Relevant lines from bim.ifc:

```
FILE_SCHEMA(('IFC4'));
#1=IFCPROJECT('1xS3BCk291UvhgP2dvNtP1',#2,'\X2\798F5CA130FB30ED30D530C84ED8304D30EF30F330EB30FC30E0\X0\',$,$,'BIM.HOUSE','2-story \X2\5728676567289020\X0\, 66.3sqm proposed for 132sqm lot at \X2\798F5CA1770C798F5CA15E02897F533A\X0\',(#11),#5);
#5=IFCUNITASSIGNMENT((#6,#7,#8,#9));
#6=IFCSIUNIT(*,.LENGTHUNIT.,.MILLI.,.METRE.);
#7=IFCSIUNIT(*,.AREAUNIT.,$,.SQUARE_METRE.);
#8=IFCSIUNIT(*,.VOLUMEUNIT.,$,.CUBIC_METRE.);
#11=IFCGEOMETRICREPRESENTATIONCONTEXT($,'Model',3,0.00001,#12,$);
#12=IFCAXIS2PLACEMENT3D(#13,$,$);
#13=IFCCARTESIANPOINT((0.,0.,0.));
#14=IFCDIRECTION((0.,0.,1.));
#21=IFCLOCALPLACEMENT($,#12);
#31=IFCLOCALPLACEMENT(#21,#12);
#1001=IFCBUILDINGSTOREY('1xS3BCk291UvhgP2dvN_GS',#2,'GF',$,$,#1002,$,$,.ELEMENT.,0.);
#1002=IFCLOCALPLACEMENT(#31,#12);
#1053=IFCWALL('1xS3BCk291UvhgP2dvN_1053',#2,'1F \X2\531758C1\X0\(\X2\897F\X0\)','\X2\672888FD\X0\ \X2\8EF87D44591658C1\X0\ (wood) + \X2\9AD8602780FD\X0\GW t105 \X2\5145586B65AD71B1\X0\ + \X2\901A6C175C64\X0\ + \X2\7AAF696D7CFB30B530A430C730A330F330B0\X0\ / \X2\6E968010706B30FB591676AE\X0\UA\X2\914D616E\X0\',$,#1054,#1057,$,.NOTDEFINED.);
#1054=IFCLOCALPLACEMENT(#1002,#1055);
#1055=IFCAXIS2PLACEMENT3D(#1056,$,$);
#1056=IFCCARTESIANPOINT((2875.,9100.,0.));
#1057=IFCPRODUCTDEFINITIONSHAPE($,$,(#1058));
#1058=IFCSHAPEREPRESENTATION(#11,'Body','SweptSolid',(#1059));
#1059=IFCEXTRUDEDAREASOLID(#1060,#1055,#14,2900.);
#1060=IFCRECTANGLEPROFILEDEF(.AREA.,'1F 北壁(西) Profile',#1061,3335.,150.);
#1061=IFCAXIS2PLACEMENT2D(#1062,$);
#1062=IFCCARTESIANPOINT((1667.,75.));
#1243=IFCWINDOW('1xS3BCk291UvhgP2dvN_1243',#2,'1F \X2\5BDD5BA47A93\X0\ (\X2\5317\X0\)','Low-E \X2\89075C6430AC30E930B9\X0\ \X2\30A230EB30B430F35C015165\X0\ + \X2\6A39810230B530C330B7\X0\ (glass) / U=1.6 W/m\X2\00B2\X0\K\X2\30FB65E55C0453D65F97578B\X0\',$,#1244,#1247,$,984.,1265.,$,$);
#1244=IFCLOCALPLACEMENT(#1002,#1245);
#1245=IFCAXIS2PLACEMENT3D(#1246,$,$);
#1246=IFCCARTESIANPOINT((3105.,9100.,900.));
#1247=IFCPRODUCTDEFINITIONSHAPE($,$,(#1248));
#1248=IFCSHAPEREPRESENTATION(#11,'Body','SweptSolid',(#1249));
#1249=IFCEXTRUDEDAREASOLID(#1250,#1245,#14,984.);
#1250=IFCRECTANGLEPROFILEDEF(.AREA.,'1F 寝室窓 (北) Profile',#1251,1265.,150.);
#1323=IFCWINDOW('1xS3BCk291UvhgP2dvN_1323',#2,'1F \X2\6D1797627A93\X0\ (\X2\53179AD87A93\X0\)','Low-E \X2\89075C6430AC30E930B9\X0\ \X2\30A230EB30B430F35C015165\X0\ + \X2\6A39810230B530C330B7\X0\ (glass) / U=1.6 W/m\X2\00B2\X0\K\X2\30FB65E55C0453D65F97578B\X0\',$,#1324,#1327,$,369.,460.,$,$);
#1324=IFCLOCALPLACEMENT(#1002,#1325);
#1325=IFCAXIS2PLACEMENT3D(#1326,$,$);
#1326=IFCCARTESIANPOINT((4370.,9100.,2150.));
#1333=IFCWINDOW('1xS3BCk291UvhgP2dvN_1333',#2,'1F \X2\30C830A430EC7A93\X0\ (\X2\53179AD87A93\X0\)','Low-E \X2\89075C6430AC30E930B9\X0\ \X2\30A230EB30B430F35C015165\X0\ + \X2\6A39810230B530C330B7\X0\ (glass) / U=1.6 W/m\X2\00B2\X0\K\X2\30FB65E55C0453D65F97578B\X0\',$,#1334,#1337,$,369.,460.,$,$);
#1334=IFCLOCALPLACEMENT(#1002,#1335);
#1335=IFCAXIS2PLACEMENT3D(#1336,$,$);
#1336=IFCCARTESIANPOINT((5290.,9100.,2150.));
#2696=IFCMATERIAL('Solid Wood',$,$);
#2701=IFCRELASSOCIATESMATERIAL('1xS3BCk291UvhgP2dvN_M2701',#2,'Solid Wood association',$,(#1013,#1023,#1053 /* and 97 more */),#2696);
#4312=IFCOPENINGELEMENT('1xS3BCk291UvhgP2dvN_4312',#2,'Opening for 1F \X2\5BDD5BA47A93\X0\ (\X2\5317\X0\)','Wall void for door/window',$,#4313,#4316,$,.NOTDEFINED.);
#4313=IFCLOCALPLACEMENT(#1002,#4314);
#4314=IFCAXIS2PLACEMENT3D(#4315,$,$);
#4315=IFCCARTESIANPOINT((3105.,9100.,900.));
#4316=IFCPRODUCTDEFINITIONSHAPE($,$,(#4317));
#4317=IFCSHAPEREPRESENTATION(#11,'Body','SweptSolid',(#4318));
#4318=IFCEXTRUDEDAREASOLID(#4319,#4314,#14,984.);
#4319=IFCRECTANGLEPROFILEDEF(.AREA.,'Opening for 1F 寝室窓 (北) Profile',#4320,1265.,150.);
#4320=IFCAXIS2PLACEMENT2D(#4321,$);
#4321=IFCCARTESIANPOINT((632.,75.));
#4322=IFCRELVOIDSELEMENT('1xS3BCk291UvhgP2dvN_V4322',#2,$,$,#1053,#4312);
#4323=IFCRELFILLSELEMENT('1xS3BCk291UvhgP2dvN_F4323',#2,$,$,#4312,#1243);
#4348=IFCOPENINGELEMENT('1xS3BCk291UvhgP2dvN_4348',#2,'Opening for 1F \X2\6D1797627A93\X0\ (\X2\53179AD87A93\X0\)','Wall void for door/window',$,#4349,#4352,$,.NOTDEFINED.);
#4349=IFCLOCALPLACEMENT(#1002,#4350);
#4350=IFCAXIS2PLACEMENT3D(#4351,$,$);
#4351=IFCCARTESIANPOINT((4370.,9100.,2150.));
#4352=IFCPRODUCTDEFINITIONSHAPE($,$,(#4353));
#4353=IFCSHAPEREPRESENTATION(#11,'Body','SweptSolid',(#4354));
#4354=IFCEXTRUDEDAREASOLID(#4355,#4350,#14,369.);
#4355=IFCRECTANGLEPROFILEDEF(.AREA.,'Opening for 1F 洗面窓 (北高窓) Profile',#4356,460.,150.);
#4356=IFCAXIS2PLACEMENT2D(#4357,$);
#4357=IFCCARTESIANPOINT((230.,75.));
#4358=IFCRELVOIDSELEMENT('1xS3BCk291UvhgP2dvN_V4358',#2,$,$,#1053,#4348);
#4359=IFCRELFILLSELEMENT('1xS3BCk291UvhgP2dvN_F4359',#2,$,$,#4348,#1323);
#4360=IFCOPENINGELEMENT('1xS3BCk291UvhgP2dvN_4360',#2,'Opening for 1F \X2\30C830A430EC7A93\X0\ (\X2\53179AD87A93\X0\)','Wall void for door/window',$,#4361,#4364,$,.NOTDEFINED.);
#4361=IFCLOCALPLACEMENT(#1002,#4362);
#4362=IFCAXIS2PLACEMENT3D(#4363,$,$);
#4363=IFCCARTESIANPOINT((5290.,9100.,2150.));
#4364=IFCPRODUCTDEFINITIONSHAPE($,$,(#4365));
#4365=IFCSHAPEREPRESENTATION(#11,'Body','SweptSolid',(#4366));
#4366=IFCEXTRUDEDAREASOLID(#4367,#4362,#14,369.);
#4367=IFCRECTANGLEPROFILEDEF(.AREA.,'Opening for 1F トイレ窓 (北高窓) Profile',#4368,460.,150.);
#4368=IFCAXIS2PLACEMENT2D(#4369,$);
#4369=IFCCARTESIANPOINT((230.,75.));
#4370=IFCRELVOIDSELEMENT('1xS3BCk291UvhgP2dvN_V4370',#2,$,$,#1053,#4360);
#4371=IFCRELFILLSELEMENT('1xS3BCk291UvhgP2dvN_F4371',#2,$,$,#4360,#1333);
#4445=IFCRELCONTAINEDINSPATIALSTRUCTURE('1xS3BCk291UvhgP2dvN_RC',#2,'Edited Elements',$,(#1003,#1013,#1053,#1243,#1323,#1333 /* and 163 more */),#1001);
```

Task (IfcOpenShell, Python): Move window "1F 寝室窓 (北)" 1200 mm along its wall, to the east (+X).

```python
import ifcopenshell
import ifcopenshell.api.geometry
import ifcopenshell.util.placement
import ifcopenshell.util.unit

model = ifcopenshell.open("bim.ifc")
unit_scale = ifcopenshell.util.unit.calculate_unit_scale(model)

window = model.by_guid("1xS3BCk291UvhgP2dvN_1243")
opening = window.FillsVoids[0].RelatingOpeningElement
wall = opening.VoidsElements[0].RelatingBuildingElement

wall_matrix = ifcopenshell.util.placement.get_local_placement(wall.ObjectPlacement)
shift = wall_matrix[:3, 0] * 1.2 / unit_scale
before = ifcopenshell.util.placement.get_local_placement(window.ObjectPlacement)[:3, 3].copy()

# The window is not placed relative to its opening, so move both.
for product in (opening, window):
    matrix = ifcopenshell.util.placement.get_local_placement(product.ObjectPlacement)
    matrix[:3, 3] += shift
    ifcopenshell.api.geometry.edit_object_placement(model, product=product, matrix=matrix, is_si=False)

after = ifcopenshell.util.placement.get_local_placement(window.ObjectPlacement)[:3, 3]
print("window moved by", (after - before).round(3) + 0.0)

model.write("bim-out.ifc")
```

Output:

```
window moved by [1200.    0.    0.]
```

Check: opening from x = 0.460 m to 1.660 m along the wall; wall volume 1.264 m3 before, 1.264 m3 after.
